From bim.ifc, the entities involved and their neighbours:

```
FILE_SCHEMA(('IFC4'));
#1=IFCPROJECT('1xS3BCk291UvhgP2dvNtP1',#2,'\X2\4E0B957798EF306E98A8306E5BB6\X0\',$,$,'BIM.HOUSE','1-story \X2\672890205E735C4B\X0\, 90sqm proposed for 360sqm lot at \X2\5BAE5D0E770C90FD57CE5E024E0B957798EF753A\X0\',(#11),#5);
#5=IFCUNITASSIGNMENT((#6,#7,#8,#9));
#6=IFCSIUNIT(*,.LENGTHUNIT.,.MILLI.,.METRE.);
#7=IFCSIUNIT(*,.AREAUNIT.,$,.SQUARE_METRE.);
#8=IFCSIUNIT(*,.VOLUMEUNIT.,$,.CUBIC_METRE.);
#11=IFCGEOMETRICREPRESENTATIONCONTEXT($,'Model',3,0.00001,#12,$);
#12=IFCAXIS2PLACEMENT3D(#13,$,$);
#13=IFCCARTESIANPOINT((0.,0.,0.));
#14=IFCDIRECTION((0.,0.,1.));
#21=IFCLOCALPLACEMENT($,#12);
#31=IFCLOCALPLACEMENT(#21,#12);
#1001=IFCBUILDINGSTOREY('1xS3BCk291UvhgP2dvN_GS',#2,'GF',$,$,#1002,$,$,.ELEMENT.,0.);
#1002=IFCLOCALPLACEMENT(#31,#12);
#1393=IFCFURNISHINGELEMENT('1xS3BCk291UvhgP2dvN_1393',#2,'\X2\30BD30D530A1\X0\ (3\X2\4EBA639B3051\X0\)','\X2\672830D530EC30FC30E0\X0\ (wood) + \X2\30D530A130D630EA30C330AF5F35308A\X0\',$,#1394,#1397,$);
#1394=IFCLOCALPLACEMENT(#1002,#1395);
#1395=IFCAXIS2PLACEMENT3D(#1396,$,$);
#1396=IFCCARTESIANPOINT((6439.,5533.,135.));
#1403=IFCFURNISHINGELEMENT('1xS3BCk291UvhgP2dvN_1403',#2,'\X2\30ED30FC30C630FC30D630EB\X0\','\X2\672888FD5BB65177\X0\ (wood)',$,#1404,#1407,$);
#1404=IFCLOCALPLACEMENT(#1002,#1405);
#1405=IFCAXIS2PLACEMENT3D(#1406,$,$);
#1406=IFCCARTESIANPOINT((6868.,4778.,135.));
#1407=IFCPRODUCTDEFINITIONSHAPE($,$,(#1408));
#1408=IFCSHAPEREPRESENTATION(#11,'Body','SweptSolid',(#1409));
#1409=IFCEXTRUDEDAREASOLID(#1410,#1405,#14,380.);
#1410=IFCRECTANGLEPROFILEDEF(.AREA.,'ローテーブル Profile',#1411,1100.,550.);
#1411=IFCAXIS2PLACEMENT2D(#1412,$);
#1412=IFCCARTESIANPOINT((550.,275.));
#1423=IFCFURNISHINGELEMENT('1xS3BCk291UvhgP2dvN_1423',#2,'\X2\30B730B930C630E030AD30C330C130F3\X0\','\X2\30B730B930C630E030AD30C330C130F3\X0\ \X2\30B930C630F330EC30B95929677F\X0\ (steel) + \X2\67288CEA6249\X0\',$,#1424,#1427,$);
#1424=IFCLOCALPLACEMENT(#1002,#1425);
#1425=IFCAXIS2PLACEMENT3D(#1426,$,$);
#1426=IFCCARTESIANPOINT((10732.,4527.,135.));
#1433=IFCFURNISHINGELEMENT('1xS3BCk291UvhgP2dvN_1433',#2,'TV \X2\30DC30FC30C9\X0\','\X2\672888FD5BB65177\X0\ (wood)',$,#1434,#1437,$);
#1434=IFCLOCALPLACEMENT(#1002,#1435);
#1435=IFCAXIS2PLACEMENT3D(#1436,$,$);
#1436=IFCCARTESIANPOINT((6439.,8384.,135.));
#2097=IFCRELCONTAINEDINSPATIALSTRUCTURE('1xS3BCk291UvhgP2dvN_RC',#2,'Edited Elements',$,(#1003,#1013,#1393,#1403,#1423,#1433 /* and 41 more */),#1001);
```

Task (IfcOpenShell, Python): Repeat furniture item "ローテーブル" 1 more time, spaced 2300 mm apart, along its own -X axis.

```python
import ifcopenshell
import ifcopenshell.api.geometry
import ifcopenshell.api.root
import ifcopenshell.util.element
import ifcopenshell.util.placement

model = ifcopenshell.open("bim.ifc")


def reuse_history(source, copy):
    """copy_class also copies each property set's owner history, people and application; keep the originals."""
    for rel in copy.IsDefinedBy:
        if rel.is_a("IfcRelDefinesByProperties") and (history := rel.RelatingPropertyDefinition.OwnerHistory):
            rel.RelatingPropertyDefinition.OwnerHistory = source.OwnerHistory
            ifcopenshell.util.element.remove_deep2(model, history)


source = model.by_guid("1xS3BCk291UvhgP2dvN_1403")
base = ifcopenshell.util.placement.get_local_placement(source.ObjectPlacement)
step = -base[:3, 0] * 2300.0

for i in range(1, 2):
    copy = ifcopenshell.api.root.copy_class(model, product=source)
    copy.Representation = ifcopenshell.util.element.copy_deep(
        model, source.Representation, exclude=["IfcGeometricRepresentationContext", "IfcRepresentationMap"]
    )
    reuse_history(source, copy)
    matrix = base.copy()
    matrix[:3, 3] += i * step
    print("added at", matrix[:3, 3].round(3) + 0.0)
    ifcopenshell.api.geometry.edit_object_placement(model, product=copy, matrix=matrix, is_si=False)

model.write("bim_edited.ifc")
```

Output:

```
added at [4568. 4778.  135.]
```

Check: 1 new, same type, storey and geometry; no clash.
